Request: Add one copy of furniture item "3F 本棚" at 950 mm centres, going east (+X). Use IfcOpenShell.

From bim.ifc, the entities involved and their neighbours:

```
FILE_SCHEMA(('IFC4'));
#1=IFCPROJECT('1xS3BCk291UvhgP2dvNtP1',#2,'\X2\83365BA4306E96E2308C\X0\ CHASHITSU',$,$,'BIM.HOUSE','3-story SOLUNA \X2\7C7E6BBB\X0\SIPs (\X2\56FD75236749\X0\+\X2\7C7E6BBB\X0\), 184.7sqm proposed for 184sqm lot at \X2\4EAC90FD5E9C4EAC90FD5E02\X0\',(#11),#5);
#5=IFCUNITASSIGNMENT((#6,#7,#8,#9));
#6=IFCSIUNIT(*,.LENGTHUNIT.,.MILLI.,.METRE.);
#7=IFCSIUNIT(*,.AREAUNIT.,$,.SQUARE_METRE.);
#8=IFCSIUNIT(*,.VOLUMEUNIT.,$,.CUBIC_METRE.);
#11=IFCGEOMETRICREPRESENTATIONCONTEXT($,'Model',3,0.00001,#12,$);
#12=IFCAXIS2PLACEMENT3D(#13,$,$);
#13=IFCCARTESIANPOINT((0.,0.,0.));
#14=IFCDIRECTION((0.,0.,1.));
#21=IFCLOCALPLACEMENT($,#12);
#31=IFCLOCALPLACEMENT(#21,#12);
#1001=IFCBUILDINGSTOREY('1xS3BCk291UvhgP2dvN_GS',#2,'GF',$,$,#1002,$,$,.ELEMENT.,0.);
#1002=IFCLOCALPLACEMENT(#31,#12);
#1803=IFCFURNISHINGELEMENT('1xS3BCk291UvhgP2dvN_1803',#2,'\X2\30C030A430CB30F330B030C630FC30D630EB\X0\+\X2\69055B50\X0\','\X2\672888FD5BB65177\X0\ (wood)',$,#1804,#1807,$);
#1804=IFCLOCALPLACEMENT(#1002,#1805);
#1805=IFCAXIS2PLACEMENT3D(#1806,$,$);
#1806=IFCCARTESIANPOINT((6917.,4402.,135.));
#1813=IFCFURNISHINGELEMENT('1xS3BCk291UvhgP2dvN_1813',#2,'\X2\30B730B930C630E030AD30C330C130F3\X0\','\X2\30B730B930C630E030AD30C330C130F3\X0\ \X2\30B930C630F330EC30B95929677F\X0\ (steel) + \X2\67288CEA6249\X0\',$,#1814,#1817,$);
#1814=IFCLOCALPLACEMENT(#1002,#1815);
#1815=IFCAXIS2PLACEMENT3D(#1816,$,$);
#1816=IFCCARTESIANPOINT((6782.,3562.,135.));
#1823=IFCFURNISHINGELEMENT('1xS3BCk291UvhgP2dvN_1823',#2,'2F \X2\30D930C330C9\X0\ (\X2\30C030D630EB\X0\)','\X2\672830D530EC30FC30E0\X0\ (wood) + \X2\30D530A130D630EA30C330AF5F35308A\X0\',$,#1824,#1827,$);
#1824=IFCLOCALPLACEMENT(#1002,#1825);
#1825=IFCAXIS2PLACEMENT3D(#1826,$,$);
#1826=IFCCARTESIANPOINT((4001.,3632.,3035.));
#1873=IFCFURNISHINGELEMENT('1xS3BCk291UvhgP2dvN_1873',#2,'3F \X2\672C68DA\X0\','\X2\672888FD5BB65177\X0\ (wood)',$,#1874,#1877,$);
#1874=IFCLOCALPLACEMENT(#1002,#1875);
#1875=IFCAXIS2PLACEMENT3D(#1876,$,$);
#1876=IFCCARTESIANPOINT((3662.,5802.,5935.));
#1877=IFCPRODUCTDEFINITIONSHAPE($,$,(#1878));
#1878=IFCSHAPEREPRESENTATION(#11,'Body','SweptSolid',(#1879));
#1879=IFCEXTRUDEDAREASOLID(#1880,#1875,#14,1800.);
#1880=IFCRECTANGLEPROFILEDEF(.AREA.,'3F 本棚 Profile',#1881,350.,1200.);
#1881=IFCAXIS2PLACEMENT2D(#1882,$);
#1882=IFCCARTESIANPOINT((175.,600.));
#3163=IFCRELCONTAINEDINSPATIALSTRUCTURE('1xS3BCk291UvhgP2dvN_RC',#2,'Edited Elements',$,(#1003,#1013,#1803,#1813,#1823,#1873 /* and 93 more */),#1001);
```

```python
import numpy as np
import ifcopenshell
import ifcopenshell.api.geometry
import ifcopenshell.api.root
import ifcopenshell.util.element
import ifcopenshell.util.placement
import ifcopenshell.util.unit

model = ifcopenshell.open("bim.ifc")
unit_scale = ifcopenshell.util.unit.calculate_unit_scale(model)


def reuse_history(source, copy):
    """copy_class also copies each property set's owner history, people and application; keep the originals."""
    for rel in copy.IsDefinedBy:
        if rel.is_a("IfcRelDefinesByProperties") and (history := rel.RelatingPropertyDefinition.OwnerHistory):
            rel.RelatingPropertyDefinition.OwnerHistory = source.OwnerHistory
            ifcopenshell.util.element.remove_deep2(model, history)


source = model.by_guid("1xS3BCk291UvhgP2dvN_1873")
base = ifcopenshell.util.placement.get_local_placement(source.ObjectPlacement)
step = np.array([1.0, 0.0, 0.0]) * 0.95 / unit_scale

for i in range(1, 2):
    copy = ifcopenshell.api.root.copy_class(model, product=source)
    copy.Representation = ifcopenshell.util.element.copy_deep(
        model, source.Representation, exclude=["IfcGeometricRepresentationContext", "IfcRepresentationMap"]
    )
    reuse_history(source, copy)
    matrix = base.copy()
    matrix[:3, 3] += i * step
    print("added at", matrix[:3, 3].round(3) + 0.0)
    ifcopenshell.api.geometry.edit_object_placement(model, product=copy, matrix=matrix, is_si=False)

model.write("bim_edited.ifc")
```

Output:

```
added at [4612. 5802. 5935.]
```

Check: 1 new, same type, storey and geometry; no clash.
